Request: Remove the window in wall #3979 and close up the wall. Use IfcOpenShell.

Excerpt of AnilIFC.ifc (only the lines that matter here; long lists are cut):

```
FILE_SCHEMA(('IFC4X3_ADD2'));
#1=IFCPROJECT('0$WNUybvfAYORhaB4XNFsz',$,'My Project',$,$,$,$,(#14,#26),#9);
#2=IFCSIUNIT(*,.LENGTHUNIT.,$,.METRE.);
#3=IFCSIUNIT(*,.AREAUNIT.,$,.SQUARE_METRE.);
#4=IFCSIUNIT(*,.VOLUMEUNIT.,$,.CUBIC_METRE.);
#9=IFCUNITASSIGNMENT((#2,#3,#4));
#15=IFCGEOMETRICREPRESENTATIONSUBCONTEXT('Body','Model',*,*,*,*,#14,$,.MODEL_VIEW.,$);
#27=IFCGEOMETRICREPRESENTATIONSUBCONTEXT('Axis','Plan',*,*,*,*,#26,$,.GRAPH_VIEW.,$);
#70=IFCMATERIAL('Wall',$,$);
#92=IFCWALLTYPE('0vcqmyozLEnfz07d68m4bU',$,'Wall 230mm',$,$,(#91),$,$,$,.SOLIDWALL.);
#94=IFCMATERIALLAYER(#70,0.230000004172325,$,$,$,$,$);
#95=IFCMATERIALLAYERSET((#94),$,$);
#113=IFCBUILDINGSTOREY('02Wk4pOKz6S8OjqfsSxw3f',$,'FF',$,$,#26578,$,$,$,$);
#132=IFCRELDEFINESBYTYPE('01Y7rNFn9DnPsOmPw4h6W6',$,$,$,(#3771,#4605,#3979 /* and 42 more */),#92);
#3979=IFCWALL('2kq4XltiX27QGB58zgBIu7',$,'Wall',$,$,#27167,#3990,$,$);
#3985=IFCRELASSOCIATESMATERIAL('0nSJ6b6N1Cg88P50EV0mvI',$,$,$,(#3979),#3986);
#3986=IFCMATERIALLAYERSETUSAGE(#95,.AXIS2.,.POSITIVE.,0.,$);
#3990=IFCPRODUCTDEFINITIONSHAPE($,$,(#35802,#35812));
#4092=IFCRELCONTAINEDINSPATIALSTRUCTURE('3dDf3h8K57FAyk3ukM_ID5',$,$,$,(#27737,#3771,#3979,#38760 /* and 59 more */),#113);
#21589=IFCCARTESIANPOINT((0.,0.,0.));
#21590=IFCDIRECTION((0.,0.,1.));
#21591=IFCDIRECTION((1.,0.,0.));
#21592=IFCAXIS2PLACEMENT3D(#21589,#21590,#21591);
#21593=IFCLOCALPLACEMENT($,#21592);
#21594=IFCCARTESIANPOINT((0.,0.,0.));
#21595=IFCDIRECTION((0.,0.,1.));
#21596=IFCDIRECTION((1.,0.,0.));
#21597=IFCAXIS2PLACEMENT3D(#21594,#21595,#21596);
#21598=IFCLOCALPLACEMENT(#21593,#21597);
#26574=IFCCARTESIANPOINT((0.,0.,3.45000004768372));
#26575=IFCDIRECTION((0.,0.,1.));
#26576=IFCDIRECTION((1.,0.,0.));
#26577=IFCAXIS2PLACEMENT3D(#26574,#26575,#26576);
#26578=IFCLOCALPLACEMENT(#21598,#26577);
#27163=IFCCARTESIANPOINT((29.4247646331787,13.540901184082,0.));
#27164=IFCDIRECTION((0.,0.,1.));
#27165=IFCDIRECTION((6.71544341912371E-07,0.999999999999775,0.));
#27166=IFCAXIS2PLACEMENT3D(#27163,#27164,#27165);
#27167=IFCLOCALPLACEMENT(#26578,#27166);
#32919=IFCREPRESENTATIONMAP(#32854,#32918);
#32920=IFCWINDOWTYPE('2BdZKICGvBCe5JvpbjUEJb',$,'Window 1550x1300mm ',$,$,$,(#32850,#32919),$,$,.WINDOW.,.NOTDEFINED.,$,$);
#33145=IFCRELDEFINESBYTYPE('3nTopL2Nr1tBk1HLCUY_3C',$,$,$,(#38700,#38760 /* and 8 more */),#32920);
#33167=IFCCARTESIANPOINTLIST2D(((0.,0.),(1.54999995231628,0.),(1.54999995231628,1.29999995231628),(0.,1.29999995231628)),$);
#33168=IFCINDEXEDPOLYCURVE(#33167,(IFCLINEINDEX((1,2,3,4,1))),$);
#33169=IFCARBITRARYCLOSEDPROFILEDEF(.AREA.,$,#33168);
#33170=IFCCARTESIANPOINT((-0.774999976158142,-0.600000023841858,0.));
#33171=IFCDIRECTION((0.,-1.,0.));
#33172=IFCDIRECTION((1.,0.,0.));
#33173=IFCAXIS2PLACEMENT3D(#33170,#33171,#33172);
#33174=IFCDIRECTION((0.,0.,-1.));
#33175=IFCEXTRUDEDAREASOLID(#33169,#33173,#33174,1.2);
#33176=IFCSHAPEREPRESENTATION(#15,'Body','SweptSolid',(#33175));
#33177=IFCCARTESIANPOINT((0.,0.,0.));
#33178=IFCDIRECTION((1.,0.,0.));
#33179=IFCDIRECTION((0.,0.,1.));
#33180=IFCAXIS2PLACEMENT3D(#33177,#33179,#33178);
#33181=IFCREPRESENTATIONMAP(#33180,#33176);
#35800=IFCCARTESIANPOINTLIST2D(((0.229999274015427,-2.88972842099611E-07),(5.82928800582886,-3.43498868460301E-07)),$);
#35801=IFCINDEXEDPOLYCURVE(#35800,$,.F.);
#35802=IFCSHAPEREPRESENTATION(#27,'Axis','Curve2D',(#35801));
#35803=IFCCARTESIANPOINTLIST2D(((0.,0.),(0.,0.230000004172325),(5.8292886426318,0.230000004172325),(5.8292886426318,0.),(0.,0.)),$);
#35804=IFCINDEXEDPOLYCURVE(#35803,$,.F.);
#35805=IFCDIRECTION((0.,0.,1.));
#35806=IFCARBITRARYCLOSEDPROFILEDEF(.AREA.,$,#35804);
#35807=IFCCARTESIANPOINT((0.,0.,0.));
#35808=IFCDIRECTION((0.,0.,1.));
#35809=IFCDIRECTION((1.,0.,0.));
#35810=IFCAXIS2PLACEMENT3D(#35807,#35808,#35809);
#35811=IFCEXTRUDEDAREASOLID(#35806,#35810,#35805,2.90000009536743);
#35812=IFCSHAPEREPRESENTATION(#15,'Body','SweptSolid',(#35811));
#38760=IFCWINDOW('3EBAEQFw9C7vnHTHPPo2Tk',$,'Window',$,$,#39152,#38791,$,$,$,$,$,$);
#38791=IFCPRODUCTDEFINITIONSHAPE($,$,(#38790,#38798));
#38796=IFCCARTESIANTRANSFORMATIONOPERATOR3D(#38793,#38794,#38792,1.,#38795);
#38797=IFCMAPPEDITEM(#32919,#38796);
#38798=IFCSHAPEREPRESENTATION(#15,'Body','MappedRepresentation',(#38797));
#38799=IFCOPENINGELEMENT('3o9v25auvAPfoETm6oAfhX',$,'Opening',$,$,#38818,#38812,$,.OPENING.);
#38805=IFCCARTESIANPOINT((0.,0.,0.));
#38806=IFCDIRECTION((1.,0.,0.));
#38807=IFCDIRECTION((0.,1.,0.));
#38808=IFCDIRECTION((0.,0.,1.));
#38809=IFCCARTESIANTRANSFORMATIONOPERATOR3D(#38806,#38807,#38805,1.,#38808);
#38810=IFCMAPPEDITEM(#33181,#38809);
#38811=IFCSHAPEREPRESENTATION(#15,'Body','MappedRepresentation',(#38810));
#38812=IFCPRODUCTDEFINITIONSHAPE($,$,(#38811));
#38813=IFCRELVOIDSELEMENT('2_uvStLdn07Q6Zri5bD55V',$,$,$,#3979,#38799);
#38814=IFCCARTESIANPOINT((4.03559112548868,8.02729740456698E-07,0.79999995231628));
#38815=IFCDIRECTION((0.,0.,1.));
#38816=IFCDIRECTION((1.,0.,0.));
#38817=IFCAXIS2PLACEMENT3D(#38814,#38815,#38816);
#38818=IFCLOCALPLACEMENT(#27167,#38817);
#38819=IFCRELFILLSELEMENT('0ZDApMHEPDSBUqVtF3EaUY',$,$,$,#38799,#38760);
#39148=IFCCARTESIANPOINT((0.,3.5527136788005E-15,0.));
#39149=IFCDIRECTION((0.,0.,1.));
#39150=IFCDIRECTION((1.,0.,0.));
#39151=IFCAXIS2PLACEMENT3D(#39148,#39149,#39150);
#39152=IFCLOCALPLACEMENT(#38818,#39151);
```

```python
import ifcopenshell
import ifcopenshell.api.feature
import ifcopenshell.api.root
import ifcopenshell.geom
import ifcopenshell.util.shape

model = ifcopenshell.open("AnilIFC.ifc")
settings = ifcopenshell.geom.settings()


def volume(element):
    """Net volume in cubic metres, openings subtracted."""
    shape = ifcopenshell.geom.create_shape(settings, element)
    return ifcopenshell.util.shape.get_volume(shape.geometry)


window = model.by_guid("3EBAEQFw9C7vnHTHPPo2Tk")
opening = window.FillsVoids[0].RelatingOpeningElement
wall = opening.VoidsElements[0].RelatingBuildingElement
before = volume(wall)

ifcopenshell.api.root.remove_product(model, product=window)
ifcopenshell.api.feature.remove_feature(model, feature=opening)

after = volume(wall)

print(f"wall volume {before:.3f} -> {after:.3f} m3")

model.write("AnilIFC-out.ifc")
```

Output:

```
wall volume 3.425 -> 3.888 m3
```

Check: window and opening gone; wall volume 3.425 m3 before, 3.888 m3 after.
